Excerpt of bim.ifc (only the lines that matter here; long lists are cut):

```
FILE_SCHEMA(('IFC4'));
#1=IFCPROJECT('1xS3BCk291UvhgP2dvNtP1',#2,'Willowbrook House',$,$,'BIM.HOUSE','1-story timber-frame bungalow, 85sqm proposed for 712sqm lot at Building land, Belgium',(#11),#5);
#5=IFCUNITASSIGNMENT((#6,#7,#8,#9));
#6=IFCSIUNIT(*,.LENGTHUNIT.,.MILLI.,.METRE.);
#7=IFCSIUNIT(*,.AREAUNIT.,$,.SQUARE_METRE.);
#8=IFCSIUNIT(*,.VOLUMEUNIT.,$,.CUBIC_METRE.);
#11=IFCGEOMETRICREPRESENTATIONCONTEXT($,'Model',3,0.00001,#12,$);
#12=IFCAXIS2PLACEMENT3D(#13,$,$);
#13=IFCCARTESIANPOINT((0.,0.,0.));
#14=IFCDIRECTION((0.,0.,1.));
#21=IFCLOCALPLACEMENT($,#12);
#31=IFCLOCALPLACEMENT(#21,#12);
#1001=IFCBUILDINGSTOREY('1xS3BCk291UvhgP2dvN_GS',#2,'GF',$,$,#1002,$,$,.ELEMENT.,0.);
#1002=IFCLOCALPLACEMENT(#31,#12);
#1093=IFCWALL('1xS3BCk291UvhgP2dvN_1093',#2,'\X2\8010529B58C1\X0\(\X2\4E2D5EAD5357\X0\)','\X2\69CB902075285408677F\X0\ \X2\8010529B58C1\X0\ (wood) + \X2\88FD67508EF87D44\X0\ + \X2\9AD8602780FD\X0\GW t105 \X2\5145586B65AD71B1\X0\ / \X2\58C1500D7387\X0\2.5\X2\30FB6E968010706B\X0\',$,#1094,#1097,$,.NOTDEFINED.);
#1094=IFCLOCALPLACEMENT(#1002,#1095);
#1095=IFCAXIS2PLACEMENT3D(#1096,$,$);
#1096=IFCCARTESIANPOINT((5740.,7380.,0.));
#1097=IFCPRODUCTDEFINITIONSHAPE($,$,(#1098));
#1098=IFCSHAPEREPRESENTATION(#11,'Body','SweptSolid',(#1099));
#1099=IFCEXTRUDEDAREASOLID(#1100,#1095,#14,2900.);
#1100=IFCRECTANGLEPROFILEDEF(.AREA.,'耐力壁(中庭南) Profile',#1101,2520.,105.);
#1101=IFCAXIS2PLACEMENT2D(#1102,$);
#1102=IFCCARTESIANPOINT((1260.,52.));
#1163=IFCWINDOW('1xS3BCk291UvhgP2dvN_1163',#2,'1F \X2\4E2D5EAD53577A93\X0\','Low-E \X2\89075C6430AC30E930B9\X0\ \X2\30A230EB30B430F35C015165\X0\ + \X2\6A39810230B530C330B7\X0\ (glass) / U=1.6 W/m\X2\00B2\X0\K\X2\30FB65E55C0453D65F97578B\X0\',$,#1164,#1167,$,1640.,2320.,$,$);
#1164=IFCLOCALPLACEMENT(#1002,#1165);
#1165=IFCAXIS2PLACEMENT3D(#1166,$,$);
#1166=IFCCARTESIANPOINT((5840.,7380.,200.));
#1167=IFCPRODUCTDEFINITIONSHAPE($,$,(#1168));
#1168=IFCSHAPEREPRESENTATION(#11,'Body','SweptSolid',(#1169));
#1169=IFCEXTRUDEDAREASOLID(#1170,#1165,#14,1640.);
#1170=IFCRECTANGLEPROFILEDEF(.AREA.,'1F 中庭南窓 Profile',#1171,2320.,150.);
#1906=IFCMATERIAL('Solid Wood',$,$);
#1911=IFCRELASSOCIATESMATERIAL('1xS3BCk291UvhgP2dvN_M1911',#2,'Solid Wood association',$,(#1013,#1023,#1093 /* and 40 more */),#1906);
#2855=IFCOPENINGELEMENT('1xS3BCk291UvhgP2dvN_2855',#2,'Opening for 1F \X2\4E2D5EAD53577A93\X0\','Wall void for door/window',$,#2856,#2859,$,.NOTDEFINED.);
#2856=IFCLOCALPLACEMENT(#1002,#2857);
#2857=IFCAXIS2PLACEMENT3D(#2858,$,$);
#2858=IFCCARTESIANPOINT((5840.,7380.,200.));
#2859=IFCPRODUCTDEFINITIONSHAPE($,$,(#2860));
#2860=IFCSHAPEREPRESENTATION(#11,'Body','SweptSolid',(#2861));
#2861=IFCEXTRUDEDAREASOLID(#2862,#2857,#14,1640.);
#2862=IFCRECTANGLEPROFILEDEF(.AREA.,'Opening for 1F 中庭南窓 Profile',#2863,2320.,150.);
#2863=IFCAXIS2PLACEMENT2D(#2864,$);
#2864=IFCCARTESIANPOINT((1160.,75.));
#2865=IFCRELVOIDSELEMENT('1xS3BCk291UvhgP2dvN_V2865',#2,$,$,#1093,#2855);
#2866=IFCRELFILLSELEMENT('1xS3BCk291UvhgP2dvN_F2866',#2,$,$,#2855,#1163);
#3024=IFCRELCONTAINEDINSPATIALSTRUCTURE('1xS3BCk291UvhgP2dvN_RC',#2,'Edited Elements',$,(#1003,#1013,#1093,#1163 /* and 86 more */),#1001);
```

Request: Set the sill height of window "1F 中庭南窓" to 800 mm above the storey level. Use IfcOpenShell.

```python
import numpy as np
import ifcopenshell
import ifcopenshell.api.geometry
import ifcopenshell.geom
import ifcopenshell.util.element
import ifcopenshell.util.placement
import ifcopenshell.util.shape
import ifcopenshell.util.unit

model = ifcopenshell.open("bim.ifc")
unit_scale = ifcopenshell.util.unit.calculate_unit_scale(model)

window = model.by_guid("1xS3BCk291UvhgP2dvN_1163")
opening = window.FillsVoids[0].RelatingOpeningElement
storey = ifcopenshell.util.element.get_container(window, ifc_class="IfcBuildingStorey")
level = ifcopenshell.util.placement.get_local_placement(storey.ObjectPlacement)[2, 3]

# The opening's origin need not be at the sill, so measure its lowest point.
shape = ifcopenshell.geom.create_shape(ifcopenshell.geom.settings(), opening)
bottom = ifcopenshell.util.shape.get_shape_bottom_elevation(shape, shape.geometry) / unit_scale
dz = level + 800.0 - bottom

shift = np.array([0.0, 0.0, dz])
# The window is not placed relative to its opening, so move both.
for product in (opening, window):
    matrix = ifcopenshell.util.placement.get_local_placement(product.ObjectPlacement)
    matrix[:3, 3] += shift
    ifcopenshell.api.geometry.edit_object_placement(model, product=product, matrix=matrix, is_si=False)

print(f"moved by {dz * unit_scale:+.3f} m")

model.write("bim_updated.ifc")
```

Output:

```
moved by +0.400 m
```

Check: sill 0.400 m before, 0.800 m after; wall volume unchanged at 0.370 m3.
